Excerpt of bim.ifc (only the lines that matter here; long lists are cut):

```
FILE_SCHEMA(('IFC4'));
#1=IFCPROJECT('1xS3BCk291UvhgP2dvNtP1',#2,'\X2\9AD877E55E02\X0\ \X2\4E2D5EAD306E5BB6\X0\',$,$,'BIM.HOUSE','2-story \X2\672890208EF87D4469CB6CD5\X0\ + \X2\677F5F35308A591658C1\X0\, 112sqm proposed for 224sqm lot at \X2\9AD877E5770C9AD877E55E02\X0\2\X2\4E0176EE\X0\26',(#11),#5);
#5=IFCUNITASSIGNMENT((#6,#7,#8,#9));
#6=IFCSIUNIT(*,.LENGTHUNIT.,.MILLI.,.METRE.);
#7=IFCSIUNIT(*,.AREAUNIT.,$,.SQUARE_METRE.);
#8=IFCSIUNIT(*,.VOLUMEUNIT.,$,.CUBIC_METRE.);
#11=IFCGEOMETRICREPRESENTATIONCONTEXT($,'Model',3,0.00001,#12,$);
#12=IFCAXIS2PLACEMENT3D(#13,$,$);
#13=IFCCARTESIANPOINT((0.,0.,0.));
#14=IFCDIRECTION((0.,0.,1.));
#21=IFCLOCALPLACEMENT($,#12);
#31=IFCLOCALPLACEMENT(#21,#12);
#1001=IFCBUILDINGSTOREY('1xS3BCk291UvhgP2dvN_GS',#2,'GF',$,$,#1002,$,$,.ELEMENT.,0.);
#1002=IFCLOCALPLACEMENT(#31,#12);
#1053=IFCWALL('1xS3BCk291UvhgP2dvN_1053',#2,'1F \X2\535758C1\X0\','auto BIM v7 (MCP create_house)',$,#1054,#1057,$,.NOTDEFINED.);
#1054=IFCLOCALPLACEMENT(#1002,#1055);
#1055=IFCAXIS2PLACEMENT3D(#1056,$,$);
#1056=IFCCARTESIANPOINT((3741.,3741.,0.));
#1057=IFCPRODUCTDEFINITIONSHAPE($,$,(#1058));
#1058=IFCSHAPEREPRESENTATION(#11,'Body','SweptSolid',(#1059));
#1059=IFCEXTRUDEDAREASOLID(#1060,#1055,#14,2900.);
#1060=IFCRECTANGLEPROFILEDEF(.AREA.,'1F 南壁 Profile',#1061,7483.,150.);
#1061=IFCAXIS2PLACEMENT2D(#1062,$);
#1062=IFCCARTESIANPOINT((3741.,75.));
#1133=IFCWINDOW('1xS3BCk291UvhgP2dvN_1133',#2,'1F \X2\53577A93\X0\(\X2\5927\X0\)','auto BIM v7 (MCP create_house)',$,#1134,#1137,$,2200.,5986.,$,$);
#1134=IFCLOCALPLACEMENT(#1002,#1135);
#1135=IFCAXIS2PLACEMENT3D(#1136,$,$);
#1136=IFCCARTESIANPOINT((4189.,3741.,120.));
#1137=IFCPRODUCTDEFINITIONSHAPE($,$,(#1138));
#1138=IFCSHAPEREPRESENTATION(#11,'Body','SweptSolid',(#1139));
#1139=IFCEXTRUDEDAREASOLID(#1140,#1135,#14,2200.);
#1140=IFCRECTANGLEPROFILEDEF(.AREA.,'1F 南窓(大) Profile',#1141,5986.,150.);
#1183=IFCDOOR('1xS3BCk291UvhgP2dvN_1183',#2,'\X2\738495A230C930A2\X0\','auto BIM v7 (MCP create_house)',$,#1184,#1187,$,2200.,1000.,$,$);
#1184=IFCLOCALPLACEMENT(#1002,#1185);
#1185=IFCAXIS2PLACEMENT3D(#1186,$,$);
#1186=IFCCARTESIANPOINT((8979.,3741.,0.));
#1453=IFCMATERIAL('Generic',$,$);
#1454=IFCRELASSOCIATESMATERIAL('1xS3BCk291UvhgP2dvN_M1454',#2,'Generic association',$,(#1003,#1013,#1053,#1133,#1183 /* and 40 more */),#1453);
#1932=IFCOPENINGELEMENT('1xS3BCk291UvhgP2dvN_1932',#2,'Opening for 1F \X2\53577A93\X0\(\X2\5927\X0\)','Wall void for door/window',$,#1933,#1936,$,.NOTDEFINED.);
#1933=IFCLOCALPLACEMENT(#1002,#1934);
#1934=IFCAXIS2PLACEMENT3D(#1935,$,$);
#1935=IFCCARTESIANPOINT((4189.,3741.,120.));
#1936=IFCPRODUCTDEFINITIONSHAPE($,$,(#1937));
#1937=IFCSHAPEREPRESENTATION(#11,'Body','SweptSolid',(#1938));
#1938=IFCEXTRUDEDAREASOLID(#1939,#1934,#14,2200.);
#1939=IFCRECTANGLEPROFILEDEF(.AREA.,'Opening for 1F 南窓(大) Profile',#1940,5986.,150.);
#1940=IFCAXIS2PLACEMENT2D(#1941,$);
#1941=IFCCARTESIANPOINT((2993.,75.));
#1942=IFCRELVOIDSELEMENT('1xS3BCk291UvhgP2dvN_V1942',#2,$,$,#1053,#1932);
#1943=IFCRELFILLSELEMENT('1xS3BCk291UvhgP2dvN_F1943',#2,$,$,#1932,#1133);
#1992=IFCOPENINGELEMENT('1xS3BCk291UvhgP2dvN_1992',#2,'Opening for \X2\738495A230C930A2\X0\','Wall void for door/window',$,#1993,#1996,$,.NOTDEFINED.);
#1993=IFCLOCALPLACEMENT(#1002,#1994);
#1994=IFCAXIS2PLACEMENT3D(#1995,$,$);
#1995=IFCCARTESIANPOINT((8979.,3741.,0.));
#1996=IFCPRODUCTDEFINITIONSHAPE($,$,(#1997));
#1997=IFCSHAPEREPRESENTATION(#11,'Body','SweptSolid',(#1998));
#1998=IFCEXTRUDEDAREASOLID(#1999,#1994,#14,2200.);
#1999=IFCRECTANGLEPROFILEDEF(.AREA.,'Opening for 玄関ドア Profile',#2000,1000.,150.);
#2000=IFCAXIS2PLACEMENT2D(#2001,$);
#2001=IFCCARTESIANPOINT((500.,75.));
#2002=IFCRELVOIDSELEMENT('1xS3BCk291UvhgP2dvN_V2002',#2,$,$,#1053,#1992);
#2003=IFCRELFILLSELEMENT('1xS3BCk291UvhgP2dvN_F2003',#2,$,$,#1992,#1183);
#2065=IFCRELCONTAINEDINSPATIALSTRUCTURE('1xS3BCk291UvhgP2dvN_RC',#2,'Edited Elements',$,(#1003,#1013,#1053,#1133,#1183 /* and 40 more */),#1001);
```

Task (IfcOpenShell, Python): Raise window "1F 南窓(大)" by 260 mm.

```python
import numpy as np
import ifcopenshell
import ifcopenshell.api.geometry
import ifcopenshell.util.placement
import ifcopenshell.util.unit

model = ifcopenshell.open("bim.ifc")
unit_scale = ifcopenshell.util.unit.calculate_unit_scale(model)

window = model.by_guid("1xS3BCk291UvhgP2dvN_1133")
opening = window.FillsVoids[0].RelatingOpeningElement
dz = 0.26 / unit_scale

shift = np.array([0.0, 0.0, dz])
# The window is not placed relative to its opening, so move both.
for product in (opening, window):
    matrix = ifcopenshell.util.placement.get_local_placement(product.ObjectPlacement)
    matrix[:3, 3] += shift
    ifcopenshell.api.geometry.edit_object_placement(model, product=product, matrix=matrix, is_si=False)

print(f"moved by {dz * unit_scale:+.3f} m")

model.write("bim_v2.ifc")
```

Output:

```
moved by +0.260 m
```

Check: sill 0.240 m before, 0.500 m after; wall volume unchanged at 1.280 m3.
